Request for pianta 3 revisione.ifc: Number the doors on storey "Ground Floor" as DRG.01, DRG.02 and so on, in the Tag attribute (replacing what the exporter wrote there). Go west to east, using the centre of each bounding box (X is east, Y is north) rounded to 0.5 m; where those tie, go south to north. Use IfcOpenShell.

First a look at what the model holds.

```python
import ifcopenshell
import ifcopenshell.util.element
import ifcopenshell.util.placement

model = ifcopenshell.open("pianta 3 revisione.ifc")
print(model.schema)
storey = next(s for s in model.by_type("IfcBuildingStorey") if s.Name == "Ground Floor")
doors = [e for e in ifcopenshell.util.element.get_decomposition(storey) if e.is_a("IfcDoor")]
for e in sorted(doors, key=lambda e: e.id()):
    origin = ifcopenshell.util.placement.get_local_placement(e.ObjectPlacement)[:3, 3]
    print(e.id(), e.Tag, e.Name, origin.round(2) + 0.0, sep=" | ")
```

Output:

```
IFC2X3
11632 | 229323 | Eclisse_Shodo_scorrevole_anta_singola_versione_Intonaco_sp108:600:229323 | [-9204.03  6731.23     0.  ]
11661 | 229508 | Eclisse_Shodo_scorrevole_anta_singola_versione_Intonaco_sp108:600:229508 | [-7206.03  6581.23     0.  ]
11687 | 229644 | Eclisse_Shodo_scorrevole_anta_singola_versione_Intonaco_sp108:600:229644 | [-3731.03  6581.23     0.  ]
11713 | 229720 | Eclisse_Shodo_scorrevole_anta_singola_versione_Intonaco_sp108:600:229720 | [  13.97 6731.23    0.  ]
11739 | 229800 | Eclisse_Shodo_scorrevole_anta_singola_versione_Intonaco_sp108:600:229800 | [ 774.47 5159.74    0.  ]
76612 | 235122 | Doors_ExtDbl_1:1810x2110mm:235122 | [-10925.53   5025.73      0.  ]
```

```python
import ifcopenshell
import ifcopenshell.geom
import ifcopenshell.util.element
import ifcopenshell.util.shape

model = ifcopenshell.open("pianta 3 revisione.ifc")
settings = ifcopenshell.geom.settings()
settings.set("use-world-coords", True)


def centre(element):
    shape = ifcopenshell.geom.create_shape(settings, element)
    return ifcopenshell.util.shape.get_bbox_centroid(shape.geometry)


storey = next(s for s in model.by_type("IfcBuildingStorey") if s.Name == "Ground Floor")
doors = [e for e in ifcopenshell.util.element.get_decomposition(storey) if e.is_a("IfcDoor")]

# Insertion points can sit at a corner or the storey origin, so sort by the geometry (in metres).
centres = {e: centre(e) for e in doors}
doors.sort(key=lambda e: (round(centres[e][0] / 0.5), centres[e][1]))

for i, e in enumerate(doors, start=1):
    number = f"DRG.{i:02d}"
    e.Tag = number
    print(e.id(), number)

model.write("pianta 3 revisione_v2.ifc")
```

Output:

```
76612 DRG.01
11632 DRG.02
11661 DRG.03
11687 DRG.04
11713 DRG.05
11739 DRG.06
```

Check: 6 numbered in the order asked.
